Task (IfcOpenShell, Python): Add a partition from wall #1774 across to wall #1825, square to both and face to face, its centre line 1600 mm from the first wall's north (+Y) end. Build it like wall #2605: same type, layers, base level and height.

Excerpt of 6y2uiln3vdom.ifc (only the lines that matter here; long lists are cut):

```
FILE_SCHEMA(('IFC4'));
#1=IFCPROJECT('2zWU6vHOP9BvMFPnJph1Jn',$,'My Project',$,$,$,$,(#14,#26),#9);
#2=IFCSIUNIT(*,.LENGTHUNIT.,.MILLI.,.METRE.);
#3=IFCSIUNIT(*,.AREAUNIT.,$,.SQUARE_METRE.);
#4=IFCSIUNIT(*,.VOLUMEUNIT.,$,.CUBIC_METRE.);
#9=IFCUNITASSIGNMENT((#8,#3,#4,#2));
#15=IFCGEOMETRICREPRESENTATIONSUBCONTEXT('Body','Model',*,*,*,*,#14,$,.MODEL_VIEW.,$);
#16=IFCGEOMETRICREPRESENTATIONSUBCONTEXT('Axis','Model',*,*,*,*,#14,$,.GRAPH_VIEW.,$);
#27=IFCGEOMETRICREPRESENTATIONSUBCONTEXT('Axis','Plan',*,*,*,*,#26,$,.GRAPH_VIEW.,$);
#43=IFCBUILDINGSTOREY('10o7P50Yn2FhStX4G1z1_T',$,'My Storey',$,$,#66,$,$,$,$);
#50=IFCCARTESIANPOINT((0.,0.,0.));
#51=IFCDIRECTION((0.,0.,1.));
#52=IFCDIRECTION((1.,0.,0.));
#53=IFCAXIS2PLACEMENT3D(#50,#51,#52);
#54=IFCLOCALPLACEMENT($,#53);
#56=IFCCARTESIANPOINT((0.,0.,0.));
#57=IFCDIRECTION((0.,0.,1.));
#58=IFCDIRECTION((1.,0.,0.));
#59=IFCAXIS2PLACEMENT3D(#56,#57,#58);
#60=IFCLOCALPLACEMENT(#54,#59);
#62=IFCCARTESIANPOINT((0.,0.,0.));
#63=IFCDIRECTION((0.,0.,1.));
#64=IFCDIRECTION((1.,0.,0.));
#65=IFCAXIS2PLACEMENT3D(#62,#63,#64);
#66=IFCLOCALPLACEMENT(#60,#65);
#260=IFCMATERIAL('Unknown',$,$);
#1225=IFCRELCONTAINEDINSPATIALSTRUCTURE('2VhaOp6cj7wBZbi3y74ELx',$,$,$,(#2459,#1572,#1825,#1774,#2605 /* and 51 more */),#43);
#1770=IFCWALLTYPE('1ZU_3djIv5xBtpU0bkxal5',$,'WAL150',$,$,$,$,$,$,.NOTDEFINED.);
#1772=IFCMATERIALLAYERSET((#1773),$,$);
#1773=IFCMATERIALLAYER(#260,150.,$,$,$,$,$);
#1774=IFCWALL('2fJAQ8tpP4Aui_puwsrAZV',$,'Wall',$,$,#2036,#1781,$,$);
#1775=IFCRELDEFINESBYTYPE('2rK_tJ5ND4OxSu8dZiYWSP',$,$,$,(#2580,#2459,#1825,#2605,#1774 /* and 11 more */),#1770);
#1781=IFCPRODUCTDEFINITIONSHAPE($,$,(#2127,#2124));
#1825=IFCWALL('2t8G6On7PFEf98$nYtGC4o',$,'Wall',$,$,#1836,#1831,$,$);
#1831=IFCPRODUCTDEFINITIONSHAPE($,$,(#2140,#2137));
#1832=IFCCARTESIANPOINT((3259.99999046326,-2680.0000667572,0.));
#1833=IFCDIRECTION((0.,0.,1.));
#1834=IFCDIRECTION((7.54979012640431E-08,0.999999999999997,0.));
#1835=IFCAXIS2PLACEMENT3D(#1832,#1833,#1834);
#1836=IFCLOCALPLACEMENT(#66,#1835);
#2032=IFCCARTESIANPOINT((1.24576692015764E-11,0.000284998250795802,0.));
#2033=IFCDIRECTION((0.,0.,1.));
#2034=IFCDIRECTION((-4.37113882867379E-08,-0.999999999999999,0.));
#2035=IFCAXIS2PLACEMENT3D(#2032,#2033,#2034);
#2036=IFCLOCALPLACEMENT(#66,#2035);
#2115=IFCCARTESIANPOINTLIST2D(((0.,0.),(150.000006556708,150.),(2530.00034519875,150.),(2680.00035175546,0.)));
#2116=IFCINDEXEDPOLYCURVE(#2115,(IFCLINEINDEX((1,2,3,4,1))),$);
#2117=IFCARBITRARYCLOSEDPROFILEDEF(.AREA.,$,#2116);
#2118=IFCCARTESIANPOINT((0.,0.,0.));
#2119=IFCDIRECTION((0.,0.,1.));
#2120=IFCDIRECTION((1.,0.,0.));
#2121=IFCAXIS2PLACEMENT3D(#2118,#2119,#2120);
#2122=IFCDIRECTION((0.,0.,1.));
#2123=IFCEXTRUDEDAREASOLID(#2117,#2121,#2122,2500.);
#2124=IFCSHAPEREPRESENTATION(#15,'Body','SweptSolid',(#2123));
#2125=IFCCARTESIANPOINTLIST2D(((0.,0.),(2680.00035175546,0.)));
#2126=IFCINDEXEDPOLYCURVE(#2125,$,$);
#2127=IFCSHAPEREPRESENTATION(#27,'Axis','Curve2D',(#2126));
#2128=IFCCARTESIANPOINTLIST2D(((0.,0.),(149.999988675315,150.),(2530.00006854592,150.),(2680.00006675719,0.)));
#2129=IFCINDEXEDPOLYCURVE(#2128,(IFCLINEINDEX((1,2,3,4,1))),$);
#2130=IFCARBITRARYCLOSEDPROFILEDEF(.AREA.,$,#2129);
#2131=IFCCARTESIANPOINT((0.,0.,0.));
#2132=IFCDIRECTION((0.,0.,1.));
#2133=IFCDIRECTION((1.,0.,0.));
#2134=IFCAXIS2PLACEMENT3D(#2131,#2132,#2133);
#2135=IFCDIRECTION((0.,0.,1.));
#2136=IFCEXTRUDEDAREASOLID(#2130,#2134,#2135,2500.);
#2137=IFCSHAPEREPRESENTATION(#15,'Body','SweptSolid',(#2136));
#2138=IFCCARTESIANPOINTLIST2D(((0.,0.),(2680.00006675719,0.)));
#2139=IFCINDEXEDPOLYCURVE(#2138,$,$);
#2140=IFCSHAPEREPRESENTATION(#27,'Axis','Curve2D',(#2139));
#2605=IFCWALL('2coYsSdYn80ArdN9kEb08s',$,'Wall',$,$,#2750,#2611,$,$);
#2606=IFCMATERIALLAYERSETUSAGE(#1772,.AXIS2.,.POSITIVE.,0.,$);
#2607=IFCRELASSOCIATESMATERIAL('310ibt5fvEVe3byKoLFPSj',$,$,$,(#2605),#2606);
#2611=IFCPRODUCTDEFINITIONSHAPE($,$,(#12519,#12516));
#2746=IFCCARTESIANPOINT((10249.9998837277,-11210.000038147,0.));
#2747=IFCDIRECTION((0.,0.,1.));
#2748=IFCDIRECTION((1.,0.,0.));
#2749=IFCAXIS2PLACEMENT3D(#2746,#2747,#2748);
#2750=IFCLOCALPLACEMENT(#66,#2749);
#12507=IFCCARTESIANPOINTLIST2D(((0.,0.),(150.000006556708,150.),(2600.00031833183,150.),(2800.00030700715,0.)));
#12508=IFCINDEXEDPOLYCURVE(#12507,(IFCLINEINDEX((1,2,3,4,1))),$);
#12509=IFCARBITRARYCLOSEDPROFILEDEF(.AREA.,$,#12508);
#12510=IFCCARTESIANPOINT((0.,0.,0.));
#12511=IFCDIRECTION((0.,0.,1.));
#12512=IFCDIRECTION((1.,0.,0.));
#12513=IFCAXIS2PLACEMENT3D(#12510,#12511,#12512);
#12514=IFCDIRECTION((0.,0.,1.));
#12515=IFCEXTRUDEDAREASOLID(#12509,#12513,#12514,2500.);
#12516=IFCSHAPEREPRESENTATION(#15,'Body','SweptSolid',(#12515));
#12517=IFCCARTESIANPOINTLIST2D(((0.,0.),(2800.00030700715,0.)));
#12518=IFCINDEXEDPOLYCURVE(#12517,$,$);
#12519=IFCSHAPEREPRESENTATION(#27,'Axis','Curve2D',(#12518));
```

```python
import numpy as np
import ifcopenshell
import ifcopenshell.api.geometry
import ifcopenshell.api.material
import ifcopenshell.api.pset
import ifcopenshell.api.root
import ifcopenshell.api.spatial
import ifcopenshell.api.type
import ifcopenshell.geom
import ifcopenshell.util.element
import ifcopenshell.util.placement
import ifcopenshell.util.representation
import ifcopenshell.util.shape
import ifcopenshell.util.unit

model = ifcopenshell.open("6y2uiln3vdom.ifc")
unit_scale = ifcopenshell.util.unit.calculate_unit_scale(model)
settings = ifcopenshell.geom.settings()
settings.set("use-world-coords", True)

start_wall = model.by_guid("2fJAQ8tpP4Aui_puwsrAZV")
end_wall = model.by_guid("2t8G6On7PFEf98$nYtGC4o")
like = model.by_guid("2coYsSdYn80ArdN9kEb08s")
matrix = ifcopenshell.util.placement.get_local_placement(start_wall.ObjectPlacement)
matrix[:3, 3] *= unit_scale


def extent(element):
    """Bounding box in the first wall's axes, in metres."""
    shape = ifcopenshell.geom.create_shape(settings, element)
    points = (ifcopenshell.util.shape.get_vertices(shape.geometry) - matrix[:3, 3]) @ matrix[:3, :3]
    return points.min(axis=0), points.max(axis=0)


y_start = extent(start_wall)[1][1]
y_end = extent(end_wall)[0][1]
like_min, like_max = extent(like)
length, height = float(abs(y_end - y_start)), float(like_max[2] - like_min[2])
layer_set = ifcopenshell.util.element.get_material(like, should_skip_usage=True)
thickness = sum(layer.LayerThickness for layer in layer_set.MaterialLayers) * unit_scale

wall = ifcopenshell.api.root.create_entity(model, ifc_class="IfcWall", name="New partition")
storey = ifcopenshell.util.element.get_container(like)
ifcopenshell.api.spatial.assign_container(model, products=[wall], relating_structure=storey)
ifcopenshell.api.type.assign_type(
    model, related_objects=[wall], relating_type=ifcopenshell.util.element.get_type(like), should_map_representations=False
)
rel = ifcopenshell.api.material.assign_material(
    model, products=[wall], type="IfcMaterialLayerSetUsage", material=layer_set
)
rel.RelatingMaterial.OffsetFromReferenceLine = -thickness / 2 / unit_scale
pset = ifcopenshell.api.pset.add_pset(model, product=wall, name="Pset_WallCommon")
ifcopenshell.api.pset.edit_pset(model, pset=pset, properties={"IsExternal": False, "LoadBearing": False})

# The axis runs down the middle of the wall.
axis = ifcopenshell.api.geometry.add_axis_representation(
    model, context=ifcopenshell.util.representation.get_context(model, "Model", "Axis"), axis=[(0.0, 0.0), (length, 0.0)]
)
body = ifcopenshell.api.geometry.add_wall_representation(
    model,
    context=ifcopenshell.util.representation.get_context(model, "Model", "Body", "MODEL_VIEW"),
    length=length,
    height=height,
    thickness=thickness,
    offset=-thickness / 2,
)
for representation in (axis, body):
    ifcopenshell.api.geometry.assign_representation(model, product=wall, representation=representation)

placement = matrix @ ifcopenshell.util.placement.rotation(90, "Z")
placement[:, 3] = matrix @ np.array([extent(start_wall)[0][0] + 1.6, y_start, like_min[2], 1.0])
ifcopenshell.api.geometry.edit_object_placement(model, product=wall, matrix=placement)

print(f"partition {length:.3f} m long, {height:.3f} m high, {thickness:.3f} m thick")

model.write("6y2uiln3vdom_updated.ifc")
```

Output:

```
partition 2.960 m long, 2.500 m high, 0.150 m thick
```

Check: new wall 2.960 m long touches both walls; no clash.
